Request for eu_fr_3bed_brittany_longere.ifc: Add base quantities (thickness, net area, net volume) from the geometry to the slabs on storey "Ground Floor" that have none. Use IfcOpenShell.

First a look at what the model holds.

```python
import ifcopenshell
import ifcopenshell.util.element
import ifcopenshell.util.unit

model = ifcopenshell.open("eu_fr_3bed_brittany_longere.ifc")
print(model.schema)
for unit_type in ("LENGTHUNIT", "AREAUNIT", "VOLUMEUNIT"):
    print(unit_type, ifcopenshell.util.unit.calculate_unit_scale(model, unit_type))
storey = next(s for s in model.by_type("IfcBuildingStorey") if s.Name == "Ground Floor")
slabs = [e for e in ifcopenshell.util.element.get_decomposition(storey) if e.is_a("IfcSlab")]
for e in sorted(slabs, key=lambda e: e.id()):
    print(e.id(), e.is_a(), e.Name, list(ifcopenshell.util.element.get_psets(e, qtos_only=True)), sep=" | ")
```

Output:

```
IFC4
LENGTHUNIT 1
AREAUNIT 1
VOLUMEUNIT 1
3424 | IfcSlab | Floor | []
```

```python
import ifcopenshell
import ifcopenshell.api.pset
import ifcopenshell.geom
import ifcopenshell.util.element
import ifcopenshell.util.shape
import ifcopenshell.util.unit

model = ifcopenshell.open("eu_fr_3bed_brittany_longere.ifc")
unit_scale = ifcopenshell.util.unit.calculate_unit_scale(model)
area_scale = ifcopenshell.util.unit.calculate_unit_scale(model, "AREAUNIT")
volume_scale = ifcopenshell.util.unit.calculate_unit_scale(model, "VOLUMEUNIT")
settings = ifcopenshell.geom.settings()

storey = next(s for s in model.by_type("IfcBuildingStorey") if s.Name == "Ground Floor")
slabs = [e for e in ifcopenshell.util.element.get_decomposition(storey) if e.is_a("IfcSlab")]

for e in sorted(slabs, key=lambda e: e.id()):
    if ifcopenshell.util.element.get_psets(e, qtos_only=True, should_inherit=False):
        continue
    # Geometry comes back in metres, in the element's own axes.
    shape = ifcopenshell.geom.create_shape(settings, e)
    values = {
        "Width": ifcopenshell.util.shape.get_z(shape.geometry) / unit_scale,
        "NetArea": ifcopenshell.util.shape.get_footprint_area(shape.geometry) / area_scale,
        "NetVolume": ifcopenshell.util.shape.get_volume(shape.geometry) / volume_scale,
    }
    qto = ifcopenshell.api.pset.add_qto(model, product=e, name="Qto_SlabBaseQuantities")
    ifcopenshell.api.pset.edit_qto(model, qto=qto, properties=values)
    print(e.id(), {k: round(v, 3) for k, v in values.items()})

model.write("eu_fr_3bed_brittany_longere_v2.ifc")
```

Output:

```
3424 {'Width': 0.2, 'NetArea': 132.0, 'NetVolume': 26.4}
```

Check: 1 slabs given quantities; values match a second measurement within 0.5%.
